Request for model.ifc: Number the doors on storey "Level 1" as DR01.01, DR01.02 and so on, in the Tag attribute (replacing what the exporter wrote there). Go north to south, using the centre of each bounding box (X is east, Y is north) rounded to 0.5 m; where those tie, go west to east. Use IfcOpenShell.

First a look at what the model holds.

```python
import ifcopenshell
import ifcopenshell.util.element
import ifcopenshell.util.placement

model = ifcopenshell.open("model.ifc")
print(model.schema)
storey = next(s for s in model.by_type("IfcBuildingStorey") if s.Name == "Level 1")
doors = [e for e in ifcopenshell.util.element.get_decomposition(storey) if e.is_a("IfcDoor")]
for e in sorted(doors, key=lambda e: e.id()):
    origin = ifcopenshell.util.placement.get_local_placement(e.ObjectPlacement)[:3, 3]
    print(e.id(), e.Tag, e.Name, origin.round(2) + 0.0, sep=" | ")
```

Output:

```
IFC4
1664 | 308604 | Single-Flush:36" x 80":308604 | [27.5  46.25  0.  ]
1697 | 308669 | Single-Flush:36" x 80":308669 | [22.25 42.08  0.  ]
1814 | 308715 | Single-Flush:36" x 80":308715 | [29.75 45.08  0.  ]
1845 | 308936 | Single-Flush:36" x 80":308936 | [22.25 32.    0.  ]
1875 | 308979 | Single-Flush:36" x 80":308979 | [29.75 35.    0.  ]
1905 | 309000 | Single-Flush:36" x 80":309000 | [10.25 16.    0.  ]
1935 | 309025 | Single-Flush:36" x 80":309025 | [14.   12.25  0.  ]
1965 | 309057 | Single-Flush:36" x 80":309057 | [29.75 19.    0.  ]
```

```python
import ifcopenshell
import ifcopenshell.geom
import ifcopenshell.util.element
import ifcopenshell.util.shape

model = ifcopenshell.open("model.ifc")
settings = ifcopenshell.geom.settings()
settings.set("use-world-coords", True)


def centre(element):
    shape = ifcopenshell.geom.create_shape(settings, element)
    return ifcopenshell.util.shape.get_bbox_centroid(shape.geometry)


storey = next(s for s in model.by_type("IfcBuildingStorey") if s.Name == "Level 1")
doors = [e for e in ifcopenshell.util.element.get_decomposition(storey) if e.is_a("IfcDoor")]

# Insertion points can sit at a corner or the storey origin, so sort by the geometry (in metres).
centres = {e: centre(e) for e in doors}
doors.sort(key=lambda e: (-round(centres[e][1] / 0.5), centres[e][0]))

for i, e in enumerate(doors, start=1):
    number = f"DR01.{i:02d}"
    e.Tag = number
    print(e.id(), number)

model.write("model_rev.ifc")
```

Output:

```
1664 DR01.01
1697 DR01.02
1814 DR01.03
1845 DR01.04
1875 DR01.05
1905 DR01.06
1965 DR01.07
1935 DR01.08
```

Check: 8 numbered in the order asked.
